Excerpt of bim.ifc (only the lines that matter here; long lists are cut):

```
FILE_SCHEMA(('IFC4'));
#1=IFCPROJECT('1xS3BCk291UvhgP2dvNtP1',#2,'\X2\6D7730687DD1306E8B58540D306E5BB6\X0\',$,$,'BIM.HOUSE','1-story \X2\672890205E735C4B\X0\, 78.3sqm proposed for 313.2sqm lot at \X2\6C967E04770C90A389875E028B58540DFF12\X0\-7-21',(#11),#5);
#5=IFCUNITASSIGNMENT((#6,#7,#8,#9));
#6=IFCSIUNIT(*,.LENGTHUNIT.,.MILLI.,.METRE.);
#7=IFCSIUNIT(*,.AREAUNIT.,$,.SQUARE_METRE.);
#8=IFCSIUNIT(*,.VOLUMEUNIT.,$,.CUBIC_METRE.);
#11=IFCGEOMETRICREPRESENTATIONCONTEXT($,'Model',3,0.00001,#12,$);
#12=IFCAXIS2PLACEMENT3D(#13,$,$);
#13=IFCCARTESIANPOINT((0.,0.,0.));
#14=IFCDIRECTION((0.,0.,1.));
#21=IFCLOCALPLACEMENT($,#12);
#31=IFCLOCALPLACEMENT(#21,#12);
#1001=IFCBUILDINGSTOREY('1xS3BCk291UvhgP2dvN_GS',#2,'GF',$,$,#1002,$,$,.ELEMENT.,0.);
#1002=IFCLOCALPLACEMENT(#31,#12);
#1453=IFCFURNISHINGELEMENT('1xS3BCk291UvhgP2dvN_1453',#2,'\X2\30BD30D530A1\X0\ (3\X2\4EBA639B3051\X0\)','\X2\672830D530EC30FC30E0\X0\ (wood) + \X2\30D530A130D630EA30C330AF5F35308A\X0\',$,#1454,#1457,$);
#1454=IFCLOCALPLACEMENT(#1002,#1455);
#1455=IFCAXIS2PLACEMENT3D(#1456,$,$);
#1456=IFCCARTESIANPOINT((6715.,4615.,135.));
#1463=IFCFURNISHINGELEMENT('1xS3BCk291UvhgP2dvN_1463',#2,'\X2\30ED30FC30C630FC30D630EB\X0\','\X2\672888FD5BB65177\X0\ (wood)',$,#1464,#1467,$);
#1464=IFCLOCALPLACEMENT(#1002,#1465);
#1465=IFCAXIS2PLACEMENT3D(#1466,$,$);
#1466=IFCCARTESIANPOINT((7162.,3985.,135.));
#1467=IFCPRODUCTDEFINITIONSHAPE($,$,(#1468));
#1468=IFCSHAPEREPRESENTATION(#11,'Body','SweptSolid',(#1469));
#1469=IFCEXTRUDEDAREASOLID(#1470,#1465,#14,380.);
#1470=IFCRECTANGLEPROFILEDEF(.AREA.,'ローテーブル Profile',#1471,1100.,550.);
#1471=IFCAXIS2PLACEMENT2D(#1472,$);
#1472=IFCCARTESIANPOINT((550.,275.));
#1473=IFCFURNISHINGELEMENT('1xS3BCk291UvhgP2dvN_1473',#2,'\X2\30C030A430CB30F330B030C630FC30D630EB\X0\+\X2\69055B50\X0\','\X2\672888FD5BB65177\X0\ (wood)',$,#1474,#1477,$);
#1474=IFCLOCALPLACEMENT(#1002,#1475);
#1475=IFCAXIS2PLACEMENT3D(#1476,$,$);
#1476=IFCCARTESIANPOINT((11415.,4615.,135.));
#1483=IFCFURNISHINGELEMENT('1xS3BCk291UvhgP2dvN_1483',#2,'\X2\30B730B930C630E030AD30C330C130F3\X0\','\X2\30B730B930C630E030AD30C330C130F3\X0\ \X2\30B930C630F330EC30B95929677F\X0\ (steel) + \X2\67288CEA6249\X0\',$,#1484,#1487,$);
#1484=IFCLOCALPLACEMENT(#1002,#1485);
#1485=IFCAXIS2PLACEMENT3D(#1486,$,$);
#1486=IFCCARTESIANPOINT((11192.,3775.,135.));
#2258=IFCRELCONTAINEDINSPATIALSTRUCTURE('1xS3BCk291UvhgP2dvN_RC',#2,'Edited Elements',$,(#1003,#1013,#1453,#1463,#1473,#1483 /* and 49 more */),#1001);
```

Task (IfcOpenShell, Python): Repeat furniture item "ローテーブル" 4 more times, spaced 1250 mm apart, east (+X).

```python
import numpy as np
import ifcopenshell
import ifcopenshell.api.geometry
import ifcopenshell.api.root
import ifcopenshell.util.element
import ifcopenshell.util.placement
import ifcopenshell.util.unit

model = ifcopenshell.open("bim.ifc")
unit_scale = ifcopenshell.util.unit.calculate_unit_scale(model)


def reuse_history(source, copy):
    """copy_class also copies each property set's owner history, people and application; keep the originals."""
    for rel in copy.IsDefinedBy:
        if rel.is_a("IfcRelDefinesByProperties") and (history := rel.RelatingPropertyDefinition.OwnerHistory):
            rel.RelatingPropertyDefinition.OwnerHistory = source.OwnerHistory
            ifcopenshell.util.element.remove_deep2(model, history)


source = model.by_guid("1xS3BCk291UvhgP2dvN_1463")
base = ifcopenshell.util.placement.get_local_placement(source.ObjectPlacement)
step = np.array([1.0, 0.0, 0.0]) * 1.25 / unit_scale

for i in range(1, 5):
    copy = ifcopenshell.api.root.copy_class(model, product=source)
    copy.Representation = ifcopenshell.util.element.copy_deep(
        model, source.Representation, exclude=["IfcGeometricRepresentationContext", "IfcRepresentationMap"]
    )
    reuse_history(source, copy)
    matrix = base.copy()
    matrix[:3, 3] += i * step
    print("added at", matrix[:3, 3].round(3) + 0.0)
    ifcopenshell.api.geometry.edit_object_placement(model, product=copy, matrix=matrix, is_si=False)

model.write("bim_updated.ifc")
```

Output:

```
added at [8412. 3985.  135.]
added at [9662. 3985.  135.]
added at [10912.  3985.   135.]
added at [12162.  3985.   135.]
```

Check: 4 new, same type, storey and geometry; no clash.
